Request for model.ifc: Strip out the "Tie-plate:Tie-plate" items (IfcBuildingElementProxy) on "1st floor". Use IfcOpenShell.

First a look at what the model holds.

```python
import ifcopenshell
import ifcopenshell.util.element

model = ifcopenshell.open("model.ifc")
print(model.schema)
storey = next(s for s in model.by_type("IfcBuildingStorey") if s.Name == "1st floor")
proxies = [e for e in ifcopenshell.util.element.get_decomposition(storey) if e.is_a("IfcBuildingElementProxy")]
seen = {}
for e in proxies:
    element_type = ifcopenshell.util.element.get_type(e)
    name = element_type.Name if element_type not in (None, e) else None
    seen[name] = seen.get(name, 0) + 1
for name, count in sorted(seen.items(), key=str):
    print(count, "x", name)
```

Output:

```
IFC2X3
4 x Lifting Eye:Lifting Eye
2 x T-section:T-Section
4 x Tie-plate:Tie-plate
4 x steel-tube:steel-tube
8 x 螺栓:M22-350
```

```python
import ifcopenshell
import ifcopenshell.api.root
import ifcopenshell.util.element

model = ifcopenshell.open("model.ifc")

storey = next(s for s in model.by_type("IfcBuildingStorey") if s.Name == "1st floor")
proxies = [e for e in ifcopenshell.util.element.get_decomposition(storey) if e.is_a("IfcBuildingElementProxy")]
targets = [e for e in proxies if (t := ifcopenshell.util.element.get_type(e)) not in (None, e) and t.Name == "Tie-plate:Tie-plate"]

for e in targets:
    ifcopenshell.api.root.remove_product(model, product=e)
print(len(targets), "removed")

model.write("model_v2.ifc")
```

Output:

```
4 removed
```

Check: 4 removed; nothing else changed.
